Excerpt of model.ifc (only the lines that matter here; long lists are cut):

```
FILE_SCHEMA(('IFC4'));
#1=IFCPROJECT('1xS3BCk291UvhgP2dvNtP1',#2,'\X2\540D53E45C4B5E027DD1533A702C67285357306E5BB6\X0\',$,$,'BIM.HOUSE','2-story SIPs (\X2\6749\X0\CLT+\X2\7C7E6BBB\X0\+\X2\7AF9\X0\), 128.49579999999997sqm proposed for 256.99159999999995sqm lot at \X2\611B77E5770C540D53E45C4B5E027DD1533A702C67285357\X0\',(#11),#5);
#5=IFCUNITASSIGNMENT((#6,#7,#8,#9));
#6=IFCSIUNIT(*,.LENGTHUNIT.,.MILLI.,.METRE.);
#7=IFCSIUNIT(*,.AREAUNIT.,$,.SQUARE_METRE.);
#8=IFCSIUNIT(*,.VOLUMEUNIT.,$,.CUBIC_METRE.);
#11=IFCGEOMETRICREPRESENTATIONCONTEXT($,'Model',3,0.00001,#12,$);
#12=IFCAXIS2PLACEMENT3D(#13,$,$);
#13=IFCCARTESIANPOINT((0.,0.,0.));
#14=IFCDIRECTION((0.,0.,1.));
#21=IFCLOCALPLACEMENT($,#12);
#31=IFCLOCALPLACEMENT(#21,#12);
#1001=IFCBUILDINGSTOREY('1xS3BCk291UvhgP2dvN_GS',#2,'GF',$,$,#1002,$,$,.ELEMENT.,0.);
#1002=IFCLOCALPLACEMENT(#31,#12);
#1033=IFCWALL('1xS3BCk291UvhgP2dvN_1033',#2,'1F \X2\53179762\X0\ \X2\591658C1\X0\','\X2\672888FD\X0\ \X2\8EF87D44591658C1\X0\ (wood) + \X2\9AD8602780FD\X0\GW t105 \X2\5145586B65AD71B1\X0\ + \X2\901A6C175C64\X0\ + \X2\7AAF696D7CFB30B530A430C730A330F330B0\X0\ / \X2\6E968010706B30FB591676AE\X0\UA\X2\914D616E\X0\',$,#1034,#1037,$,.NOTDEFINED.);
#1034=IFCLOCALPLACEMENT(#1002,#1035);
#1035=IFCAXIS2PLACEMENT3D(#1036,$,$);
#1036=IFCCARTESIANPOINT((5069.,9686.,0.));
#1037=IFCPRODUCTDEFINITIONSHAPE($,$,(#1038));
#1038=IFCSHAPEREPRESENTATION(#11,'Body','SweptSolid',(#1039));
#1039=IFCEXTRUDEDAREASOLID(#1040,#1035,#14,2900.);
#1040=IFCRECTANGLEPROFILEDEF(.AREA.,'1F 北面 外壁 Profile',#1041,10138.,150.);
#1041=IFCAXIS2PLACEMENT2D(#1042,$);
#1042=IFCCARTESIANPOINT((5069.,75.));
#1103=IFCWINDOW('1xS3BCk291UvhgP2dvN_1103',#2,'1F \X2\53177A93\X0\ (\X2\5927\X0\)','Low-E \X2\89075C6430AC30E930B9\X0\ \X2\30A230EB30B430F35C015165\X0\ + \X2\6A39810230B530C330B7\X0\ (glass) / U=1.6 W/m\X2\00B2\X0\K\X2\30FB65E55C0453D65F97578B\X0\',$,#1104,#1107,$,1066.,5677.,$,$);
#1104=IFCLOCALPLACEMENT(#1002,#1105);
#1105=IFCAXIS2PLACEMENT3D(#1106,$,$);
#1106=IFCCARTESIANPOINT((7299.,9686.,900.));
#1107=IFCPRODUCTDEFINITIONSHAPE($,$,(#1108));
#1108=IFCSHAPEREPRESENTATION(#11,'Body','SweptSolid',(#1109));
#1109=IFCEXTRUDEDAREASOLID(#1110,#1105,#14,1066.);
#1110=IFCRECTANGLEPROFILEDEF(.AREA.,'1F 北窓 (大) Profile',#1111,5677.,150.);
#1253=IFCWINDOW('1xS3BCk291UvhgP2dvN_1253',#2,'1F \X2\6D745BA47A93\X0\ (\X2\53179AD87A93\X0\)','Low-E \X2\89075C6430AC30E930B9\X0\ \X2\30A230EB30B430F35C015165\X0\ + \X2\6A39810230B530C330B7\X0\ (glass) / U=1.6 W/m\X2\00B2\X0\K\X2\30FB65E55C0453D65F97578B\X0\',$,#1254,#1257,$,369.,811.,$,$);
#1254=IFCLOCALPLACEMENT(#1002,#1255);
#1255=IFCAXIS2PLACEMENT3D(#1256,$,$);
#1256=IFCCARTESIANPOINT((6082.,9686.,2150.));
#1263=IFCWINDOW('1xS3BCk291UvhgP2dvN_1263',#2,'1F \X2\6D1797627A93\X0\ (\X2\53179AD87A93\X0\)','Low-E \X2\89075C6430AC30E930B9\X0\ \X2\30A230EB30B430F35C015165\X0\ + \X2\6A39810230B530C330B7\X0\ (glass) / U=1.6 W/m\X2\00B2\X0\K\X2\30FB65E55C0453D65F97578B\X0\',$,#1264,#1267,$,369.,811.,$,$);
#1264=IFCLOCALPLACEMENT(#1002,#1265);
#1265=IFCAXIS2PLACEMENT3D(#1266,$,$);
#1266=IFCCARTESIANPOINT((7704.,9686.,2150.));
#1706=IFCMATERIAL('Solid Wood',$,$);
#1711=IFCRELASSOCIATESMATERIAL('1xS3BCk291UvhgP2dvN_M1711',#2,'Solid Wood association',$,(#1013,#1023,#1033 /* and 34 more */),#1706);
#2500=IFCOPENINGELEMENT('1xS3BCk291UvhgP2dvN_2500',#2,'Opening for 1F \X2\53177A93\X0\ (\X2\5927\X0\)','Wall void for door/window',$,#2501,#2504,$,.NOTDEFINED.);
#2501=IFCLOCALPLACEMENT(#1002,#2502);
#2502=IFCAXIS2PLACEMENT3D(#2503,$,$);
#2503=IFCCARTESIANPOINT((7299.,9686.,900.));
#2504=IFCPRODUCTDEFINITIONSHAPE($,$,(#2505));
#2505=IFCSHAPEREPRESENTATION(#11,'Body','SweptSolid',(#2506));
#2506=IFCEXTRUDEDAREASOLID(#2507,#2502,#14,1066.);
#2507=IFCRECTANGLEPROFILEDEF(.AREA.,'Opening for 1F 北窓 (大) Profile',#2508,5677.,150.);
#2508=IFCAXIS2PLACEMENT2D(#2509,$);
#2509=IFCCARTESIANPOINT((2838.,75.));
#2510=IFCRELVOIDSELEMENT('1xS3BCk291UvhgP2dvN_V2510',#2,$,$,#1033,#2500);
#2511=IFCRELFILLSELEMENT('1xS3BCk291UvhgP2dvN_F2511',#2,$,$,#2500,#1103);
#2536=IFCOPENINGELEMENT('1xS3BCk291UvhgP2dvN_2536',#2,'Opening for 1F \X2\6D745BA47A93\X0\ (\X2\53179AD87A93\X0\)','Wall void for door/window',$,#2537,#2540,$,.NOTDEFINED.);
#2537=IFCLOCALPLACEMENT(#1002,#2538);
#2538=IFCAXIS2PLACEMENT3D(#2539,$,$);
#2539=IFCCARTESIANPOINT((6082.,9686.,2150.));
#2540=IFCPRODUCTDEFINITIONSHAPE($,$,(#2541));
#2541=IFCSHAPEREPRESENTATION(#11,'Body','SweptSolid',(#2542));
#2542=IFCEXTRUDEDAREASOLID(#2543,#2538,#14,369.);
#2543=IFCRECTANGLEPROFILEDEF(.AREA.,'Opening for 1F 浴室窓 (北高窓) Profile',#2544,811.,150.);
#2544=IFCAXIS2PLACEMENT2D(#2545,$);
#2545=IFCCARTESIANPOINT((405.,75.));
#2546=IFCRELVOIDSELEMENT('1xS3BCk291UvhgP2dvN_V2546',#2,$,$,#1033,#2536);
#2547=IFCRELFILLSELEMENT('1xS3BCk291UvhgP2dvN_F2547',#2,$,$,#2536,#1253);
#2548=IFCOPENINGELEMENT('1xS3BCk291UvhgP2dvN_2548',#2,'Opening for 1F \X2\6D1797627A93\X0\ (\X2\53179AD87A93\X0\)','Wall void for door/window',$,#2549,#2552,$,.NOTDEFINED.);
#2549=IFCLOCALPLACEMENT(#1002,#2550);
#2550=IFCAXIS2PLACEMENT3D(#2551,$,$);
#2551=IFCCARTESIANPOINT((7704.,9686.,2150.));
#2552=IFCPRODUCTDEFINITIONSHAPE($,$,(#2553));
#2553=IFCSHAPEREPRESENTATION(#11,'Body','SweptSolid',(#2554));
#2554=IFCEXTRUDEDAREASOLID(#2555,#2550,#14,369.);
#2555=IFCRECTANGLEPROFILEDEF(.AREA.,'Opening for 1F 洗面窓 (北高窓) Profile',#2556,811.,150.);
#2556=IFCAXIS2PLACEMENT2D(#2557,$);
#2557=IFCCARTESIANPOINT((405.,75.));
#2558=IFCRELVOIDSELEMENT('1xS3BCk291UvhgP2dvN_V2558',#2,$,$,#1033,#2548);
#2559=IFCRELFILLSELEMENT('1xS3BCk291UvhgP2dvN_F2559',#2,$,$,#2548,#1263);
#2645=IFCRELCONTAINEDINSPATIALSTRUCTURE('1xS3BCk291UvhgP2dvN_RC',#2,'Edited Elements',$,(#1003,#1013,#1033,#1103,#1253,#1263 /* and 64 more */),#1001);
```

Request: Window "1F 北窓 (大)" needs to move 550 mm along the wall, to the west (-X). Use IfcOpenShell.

```python
import ifcopenshell
import ifcopenshell.api.geometry
import ifcopenshell.util.placement

model = ifcopenshell.open("model.ifc")

window = model.by_guid("1xS3BCk291UvhgP2dvN_1103")
opening = window.FillsVoids[0].RelatingOpeningElement
wall = opening.VoidsElements[0].RelatingBuildingElement

wall_matrix = ifcopenshell.util.placement.get_local_placement(wall.ObjectPlacement)
shift = wall_matrix[:3, 0] * -550.0
before = ifcopenshell.util.placement.get_local_placement(window.ObjectPlacement)[:3, 3].copy()

# The window is not placed relative to its opening, so move both.
for product in (opening, window):
    matrix = ifcopenshell.util.placement.get_local_placement(product.ObjectPlacement)
    matrix[:3, 3] += shift
    ifcopenshell.api.geometry.edit_object_placement(model, product=product, matrix=matrix, is_si=False)

after = ifcopenshell.util.placement.get_local_placement(window.ObjectPlacement)[:3, 3]
print("window moved by", (after - before).round(3) + 0.0)

model.write("model_edited.ifc")
```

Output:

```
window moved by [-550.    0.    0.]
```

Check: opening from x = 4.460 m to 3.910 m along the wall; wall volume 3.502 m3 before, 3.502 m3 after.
